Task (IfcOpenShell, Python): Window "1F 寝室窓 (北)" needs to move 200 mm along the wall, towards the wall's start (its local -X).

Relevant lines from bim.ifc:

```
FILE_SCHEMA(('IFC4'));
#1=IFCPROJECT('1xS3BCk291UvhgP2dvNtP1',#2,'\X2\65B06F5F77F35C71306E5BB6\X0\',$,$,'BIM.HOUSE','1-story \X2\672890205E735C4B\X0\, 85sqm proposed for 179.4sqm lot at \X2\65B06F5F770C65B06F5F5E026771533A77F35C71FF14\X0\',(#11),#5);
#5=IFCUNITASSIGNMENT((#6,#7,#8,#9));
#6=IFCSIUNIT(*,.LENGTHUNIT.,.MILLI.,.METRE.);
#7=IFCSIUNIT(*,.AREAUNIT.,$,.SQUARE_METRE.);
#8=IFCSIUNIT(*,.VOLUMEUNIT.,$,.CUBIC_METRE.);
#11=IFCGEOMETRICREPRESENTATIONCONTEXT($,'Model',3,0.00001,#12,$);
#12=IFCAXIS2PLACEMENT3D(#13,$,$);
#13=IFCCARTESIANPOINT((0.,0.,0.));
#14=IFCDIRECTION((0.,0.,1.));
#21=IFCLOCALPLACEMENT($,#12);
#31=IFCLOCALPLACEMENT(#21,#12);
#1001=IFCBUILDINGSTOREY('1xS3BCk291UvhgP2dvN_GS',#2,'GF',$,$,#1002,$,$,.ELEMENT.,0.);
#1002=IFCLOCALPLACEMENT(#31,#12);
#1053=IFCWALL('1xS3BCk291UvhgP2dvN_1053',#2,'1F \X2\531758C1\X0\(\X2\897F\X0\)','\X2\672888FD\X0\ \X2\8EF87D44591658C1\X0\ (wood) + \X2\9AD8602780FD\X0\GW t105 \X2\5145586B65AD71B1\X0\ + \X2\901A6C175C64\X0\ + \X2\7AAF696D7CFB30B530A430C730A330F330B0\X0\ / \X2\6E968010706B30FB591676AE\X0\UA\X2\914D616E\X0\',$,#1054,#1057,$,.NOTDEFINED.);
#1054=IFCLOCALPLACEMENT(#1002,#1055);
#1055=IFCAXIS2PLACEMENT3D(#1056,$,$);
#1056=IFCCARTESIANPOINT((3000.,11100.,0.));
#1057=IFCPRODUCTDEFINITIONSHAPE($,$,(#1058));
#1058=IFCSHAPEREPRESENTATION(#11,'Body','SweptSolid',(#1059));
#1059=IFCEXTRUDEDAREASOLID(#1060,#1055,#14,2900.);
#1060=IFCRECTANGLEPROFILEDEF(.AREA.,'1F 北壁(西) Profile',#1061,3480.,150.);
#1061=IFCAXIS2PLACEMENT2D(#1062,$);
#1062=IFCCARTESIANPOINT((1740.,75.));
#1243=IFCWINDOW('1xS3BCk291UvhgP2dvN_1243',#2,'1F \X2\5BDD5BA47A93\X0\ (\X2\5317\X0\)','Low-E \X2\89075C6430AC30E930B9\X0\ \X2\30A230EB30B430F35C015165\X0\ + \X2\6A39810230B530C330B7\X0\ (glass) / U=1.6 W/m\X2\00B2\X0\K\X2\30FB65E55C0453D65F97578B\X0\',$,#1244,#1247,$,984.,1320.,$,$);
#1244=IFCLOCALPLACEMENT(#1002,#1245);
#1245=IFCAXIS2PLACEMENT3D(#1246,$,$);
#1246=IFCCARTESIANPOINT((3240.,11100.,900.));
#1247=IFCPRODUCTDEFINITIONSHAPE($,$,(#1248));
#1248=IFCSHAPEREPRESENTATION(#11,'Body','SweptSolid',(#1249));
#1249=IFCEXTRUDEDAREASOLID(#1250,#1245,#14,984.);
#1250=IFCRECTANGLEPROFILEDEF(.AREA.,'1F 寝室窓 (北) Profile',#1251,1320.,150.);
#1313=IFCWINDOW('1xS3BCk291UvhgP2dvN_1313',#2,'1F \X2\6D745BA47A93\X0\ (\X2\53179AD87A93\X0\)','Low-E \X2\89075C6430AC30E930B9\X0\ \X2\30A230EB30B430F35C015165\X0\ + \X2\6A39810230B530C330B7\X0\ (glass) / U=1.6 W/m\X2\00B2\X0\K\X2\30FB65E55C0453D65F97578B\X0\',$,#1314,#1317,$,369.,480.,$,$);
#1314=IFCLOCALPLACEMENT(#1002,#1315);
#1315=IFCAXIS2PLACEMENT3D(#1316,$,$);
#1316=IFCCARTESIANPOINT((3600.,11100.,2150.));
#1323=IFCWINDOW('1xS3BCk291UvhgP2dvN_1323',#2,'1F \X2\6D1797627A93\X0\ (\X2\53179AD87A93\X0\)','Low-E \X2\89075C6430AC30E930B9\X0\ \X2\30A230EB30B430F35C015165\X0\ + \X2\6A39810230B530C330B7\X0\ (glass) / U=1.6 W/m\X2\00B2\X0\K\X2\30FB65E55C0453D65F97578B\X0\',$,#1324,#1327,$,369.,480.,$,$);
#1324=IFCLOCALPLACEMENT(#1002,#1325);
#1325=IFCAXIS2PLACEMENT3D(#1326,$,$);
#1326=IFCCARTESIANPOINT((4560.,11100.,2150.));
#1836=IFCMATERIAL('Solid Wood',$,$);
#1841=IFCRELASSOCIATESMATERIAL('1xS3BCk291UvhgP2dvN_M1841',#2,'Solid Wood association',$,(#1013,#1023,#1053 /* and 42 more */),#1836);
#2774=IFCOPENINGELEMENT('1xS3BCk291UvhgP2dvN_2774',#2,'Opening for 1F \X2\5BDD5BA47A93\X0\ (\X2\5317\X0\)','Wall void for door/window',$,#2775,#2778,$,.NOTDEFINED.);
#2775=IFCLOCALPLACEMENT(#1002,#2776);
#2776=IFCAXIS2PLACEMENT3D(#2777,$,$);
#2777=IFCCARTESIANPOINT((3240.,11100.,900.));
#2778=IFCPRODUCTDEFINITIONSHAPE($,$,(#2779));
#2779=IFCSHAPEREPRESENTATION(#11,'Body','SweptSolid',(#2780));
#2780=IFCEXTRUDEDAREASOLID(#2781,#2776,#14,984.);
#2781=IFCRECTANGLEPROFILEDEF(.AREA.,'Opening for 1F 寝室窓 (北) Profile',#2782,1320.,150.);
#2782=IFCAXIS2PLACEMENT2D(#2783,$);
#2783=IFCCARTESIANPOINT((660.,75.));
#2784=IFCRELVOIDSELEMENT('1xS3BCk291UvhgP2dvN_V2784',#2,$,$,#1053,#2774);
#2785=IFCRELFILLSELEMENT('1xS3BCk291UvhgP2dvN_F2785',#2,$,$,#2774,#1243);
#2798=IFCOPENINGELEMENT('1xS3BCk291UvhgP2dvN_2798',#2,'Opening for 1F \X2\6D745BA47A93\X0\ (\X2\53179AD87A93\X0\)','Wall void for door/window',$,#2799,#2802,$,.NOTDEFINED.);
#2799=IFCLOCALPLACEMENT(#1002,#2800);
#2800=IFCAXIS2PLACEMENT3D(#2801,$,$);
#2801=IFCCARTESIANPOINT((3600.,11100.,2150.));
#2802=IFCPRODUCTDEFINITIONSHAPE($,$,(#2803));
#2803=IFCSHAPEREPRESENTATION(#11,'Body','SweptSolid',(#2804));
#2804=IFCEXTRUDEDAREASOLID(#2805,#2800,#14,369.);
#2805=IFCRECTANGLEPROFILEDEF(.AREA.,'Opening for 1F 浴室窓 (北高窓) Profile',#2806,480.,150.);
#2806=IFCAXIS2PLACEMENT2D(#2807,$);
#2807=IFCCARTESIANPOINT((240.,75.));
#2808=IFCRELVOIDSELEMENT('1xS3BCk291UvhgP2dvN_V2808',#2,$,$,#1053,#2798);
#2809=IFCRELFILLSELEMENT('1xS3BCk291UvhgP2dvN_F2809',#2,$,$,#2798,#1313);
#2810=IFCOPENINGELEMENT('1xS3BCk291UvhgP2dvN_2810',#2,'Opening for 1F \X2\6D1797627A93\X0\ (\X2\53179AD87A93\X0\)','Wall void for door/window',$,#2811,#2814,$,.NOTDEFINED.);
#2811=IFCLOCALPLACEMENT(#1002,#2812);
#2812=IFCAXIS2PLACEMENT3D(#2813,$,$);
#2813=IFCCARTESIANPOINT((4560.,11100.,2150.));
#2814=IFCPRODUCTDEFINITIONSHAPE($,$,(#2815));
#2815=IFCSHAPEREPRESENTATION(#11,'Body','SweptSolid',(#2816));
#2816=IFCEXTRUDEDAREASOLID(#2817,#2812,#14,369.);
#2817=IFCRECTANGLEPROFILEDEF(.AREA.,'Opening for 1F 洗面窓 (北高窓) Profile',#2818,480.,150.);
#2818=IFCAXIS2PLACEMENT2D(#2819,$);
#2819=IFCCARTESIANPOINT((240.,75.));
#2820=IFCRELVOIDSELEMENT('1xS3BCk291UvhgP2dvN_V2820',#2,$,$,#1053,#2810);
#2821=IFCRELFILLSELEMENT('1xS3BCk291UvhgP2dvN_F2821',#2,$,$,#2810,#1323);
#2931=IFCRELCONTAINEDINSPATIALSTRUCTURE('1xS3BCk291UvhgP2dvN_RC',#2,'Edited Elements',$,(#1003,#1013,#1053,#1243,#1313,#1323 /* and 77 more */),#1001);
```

```python
import ifcopenshell
import ifcopenshell.api.geometry
import ifcopenshell.util.placement
import ifcopenshell.util.unit

model = ifcopenshell.open("bim.ifc")
unit_scale = ifcopenshell.util.unit.calculate_unit_scale(model)

window = model.by_guid("1xS3BCk291UvhgP2dvN_1243")
opening = window.FillsVoids[0].RelatingOpeningElement
wall = opening.VoidsElements[0].RelatingBuildingElement

wall_matrix = ifcopenshell.util.placement.get_local_placement(wall.ObjectPlacement)
shift = wall_matrix[:3, 0] * -0.2 / unit_scale
before = ifcopenshell.util.placement.get_local_placement(window.ObjectPlacement)[:3, 3].copy()

# The window is not placed relative to its opening, so move both.
for product in (opening, window):
    matrix = ifcopenshell.util.placement.get_local_placement(product.ObjectPlacement)
    matrix[:3, 3] += shift
    ifcopenshell.api.geometry.edit_object_placement(model, product=product, matrix=matrix, is_si=False)

after = ifcopenshell.util.placement.get_local_placement(window.ObjectPlacement)[:3, 3]
print("window moved by", (after - before).round(3) + 0.0)

model.write("bim_v2.ifc")
```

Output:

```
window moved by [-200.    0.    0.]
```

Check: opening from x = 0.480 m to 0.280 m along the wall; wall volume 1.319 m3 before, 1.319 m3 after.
